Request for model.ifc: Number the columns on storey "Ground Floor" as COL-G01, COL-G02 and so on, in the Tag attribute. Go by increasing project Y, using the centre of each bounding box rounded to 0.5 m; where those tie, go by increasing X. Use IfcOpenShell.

First a look at what the model holds.

```python
import ifcopenshell
import ifcopenshell.util.element
import ifcopenshell.util.placement

model = ifcopenshell.open("model.ifc")
print(model.schema)
storey = next(s for s in model.by_type("IfcBuildingStorey") if s.Name == "Ground Floor")
columns = [e for e in ifcopenshell.util.element.get_decomposition(storey) if e.is_a("IfcColumn")]
for e in sorted(columns, key=lambda e: e.id()):
    origin = ifcopenshell.util.placement.get_local_placement(e.ObjectPlacement)[:3, 3]
    print(e.id(), e.Tag, e.Name, origin.round(2) + 0.0, sep=" | ")
```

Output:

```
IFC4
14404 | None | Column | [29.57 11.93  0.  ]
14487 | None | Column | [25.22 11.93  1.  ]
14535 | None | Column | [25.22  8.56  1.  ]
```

```python
import ifcopenshell
import ifcopenshell.geom
import ifcopenshell.util.element
import ifcopenshell.util.shape

model = ifcopenshell.open("model.ifc")
settings = ifcopenshell.geom.settings()
settings.set("use-world-coords", True)


def centre(element):
    shape = ifcopenshell.geom.create_shape(settings, element)
    return ifcopenshell.util.shape.get_bbox_centroid(shape.geometry)


storey = next(s for s in model.by_type("IfcBuildingStorey") if s.Name == "Ground Floor")
columns = [e for e in ifcopenshell.util.element.get_decomposition(storey) if e.is_a("IfcColumn")]

# Insertion points can sit at a corner or the storey origin, so sort by the geometry (in metres).
centres = {e: centre(e) for e in columns}
columns.sort(key=lambda e: (round(centres[e][1] / 0.5), centres[e][0]))

for i, e in enumerate(columns, start=1):
    number = f"COL-G{i:02d}"
    e.Tag = number
    print(e.id(), number)

model.write("model_edited.ifc")
```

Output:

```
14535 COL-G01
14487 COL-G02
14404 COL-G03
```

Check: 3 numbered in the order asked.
